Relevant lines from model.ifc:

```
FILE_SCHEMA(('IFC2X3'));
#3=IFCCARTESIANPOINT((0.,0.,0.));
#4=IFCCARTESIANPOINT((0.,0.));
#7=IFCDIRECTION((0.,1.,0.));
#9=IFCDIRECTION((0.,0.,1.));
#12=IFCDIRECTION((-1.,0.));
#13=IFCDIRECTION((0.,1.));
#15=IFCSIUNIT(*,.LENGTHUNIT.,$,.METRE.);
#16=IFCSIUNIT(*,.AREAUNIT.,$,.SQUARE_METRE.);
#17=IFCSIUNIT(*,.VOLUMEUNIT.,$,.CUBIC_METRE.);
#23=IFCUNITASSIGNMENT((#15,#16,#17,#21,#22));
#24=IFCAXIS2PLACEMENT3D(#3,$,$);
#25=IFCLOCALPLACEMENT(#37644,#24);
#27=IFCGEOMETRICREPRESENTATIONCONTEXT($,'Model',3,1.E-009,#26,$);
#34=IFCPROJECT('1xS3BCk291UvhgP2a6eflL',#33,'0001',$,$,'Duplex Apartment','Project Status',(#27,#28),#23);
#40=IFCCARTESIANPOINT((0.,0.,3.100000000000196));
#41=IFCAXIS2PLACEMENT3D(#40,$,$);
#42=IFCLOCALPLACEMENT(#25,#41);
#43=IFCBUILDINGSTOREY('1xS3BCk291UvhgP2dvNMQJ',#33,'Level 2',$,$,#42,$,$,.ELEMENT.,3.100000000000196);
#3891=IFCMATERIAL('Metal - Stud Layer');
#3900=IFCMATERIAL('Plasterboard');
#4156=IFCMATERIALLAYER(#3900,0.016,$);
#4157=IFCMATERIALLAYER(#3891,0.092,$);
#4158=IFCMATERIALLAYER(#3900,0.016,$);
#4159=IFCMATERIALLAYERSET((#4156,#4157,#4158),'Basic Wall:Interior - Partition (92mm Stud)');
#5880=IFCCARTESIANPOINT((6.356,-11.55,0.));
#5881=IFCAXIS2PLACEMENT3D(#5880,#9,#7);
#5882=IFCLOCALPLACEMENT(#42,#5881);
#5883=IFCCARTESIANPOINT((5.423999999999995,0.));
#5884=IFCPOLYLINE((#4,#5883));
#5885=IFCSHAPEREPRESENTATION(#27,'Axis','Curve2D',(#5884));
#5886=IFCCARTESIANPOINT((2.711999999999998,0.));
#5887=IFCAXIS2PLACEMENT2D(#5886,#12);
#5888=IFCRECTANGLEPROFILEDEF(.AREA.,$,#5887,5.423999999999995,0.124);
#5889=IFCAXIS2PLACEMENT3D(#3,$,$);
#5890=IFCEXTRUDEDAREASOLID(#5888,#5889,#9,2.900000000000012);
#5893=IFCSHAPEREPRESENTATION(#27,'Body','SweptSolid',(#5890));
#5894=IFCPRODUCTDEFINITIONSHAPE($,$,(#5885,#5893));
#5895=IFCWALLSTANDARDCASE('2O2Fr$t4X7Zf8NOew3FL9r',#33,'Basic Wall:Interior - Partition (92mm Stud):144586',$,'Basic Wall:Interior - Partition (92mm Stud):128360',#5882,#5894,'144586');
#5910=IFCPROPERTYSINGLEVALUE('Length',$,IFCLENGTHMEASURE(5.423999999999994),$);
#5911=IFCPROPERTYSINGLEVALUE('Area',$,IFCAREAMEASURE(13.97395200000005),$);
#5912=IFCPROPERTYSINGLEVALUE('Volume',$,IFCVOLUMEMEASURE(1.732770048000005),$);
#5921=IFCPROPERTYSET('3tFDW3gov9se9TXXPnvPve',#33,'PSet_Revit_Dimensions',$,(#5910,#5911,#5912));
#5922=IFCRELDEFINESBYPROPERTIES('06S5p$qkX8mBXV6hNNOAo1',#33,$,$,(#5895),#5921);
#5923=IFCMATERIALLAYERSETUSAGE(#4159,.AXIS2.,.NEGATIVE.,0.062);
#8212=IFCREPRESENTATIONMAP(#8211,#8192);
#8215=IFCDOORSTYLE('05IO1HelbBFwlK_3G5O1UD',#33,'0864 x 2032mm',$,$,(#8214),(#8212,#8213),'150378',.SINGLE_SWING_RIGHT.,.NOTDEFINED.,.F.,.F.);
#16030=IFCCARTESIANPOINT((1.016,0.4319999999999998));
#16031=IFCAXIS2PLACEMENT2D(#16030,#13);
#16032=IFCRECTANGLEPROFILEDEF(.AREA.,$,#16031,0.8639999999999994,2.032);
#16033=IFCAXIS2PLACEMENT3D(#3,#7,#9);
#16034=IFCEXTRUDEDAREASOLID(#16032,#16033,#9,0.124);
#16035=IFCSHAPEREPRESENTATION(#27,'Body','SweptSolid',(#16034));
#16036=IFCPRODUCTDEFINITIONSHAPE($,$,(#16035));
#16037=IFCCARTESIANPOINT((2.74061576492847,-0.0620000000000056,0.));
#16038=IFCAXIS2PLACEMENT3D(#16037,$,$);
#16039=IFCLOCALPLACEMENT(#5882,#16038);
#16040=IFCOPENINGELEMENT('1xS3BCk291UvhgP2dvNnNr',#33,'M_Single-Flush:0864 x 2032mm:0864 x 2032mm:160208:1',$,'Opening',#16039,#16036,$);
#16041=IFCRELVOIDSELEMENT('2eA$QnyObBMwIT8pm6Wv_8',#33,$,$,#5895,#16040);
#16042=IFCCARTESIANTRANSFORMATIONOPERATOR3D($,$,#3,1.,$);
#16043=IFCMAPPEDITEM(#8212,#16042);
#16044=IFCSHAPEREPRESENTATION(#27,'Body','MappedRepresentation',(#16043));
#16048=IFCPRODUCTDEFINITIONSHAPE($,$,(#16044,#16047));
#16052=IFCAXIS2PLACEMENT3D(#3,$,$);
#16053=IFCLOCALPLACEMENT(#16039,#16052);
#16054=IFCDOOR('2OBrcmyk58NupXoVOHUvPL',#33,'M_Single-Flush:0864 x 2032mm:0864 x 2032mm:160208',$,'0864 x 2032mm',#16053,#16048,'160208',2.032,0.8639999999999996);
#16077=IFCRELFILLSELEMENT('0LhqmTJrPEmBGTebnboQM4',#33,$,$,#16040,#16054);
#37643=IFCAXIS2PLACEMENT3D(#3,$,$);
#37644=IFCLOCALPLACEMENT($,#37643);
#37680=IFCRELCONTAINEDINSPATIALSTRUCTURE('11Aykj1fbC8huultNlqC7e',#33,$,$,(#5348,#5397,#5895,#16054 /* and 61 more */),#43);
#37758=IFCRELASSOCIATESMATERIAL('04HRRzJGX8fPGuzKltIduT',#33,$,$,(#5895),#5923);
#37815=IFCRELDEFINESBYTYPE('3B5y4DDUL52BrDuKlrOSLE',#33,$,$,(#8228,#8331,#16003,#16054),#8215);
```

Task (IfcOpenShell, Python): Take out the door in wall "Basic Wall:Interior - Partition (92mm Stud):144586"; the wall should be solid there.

```python
import ifcopenshell
import ifcopenshell.api.feature
import ifcopenshell.api.pset
import ifcopenshell.api.root
import ifcopenshell.geom
import ifcopenshell.util.element
import ifcopenshell.util.shape
import ifcopenshell.util.unit

model = ifcopenshell.open("model.ifc")
area_scale = ifcopenshell.util.unit.calculate_unit_scale(model, "AREAUNIT")
volume_scale = ifcopenshell.util.unit.calculate_unit_scale(model, "VOLUMEUNIT")
settings = ifcopenshell.geom.settings()


def volume(element):
    """Net volume in cubic metres, openings subtracted."""
    shape = ifcopenshell.geom.create_shape(settings, element)
    return ifcopenshell.util.shape.get_volume(shape.geometry)


door = model.by_id(16054)
opening = door.FillsVoids[0].RelatingOpeningElement
wall = opening.VoidsElements[0].RelatingBuildingElement
before = volume(wall)

ifcopenshell.api.root.remove_product(model, product=door)
ifcopenshell.api.feature.remove_feature(model, feature=opening)

after = volume(wall)
thickness = 0.124  # wall thickness in metres

# Update the wall's stored quantities.
pset = model.by_id(ifcopenshell.util.element.get_pset(wall, "PSet_Revit_Dimensions", should_inherit=False)["id"])
ifcopenshell.api.pset.edit_pset(model, pset=pset, properties={
    "Area": model.create_entity("IfcAreaMeasure", after / thickness / area_scale),
    "Volume": model.create_entity("IfcVolumeMeasure", after / volume_scale),
})

print(f"wall volume {before:.3f} -> {after:.3f} m3")

model.write("model_edited.ifc")
```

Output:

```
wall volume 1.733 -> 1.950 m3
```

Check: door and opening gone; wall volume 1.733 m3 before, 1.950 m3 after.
